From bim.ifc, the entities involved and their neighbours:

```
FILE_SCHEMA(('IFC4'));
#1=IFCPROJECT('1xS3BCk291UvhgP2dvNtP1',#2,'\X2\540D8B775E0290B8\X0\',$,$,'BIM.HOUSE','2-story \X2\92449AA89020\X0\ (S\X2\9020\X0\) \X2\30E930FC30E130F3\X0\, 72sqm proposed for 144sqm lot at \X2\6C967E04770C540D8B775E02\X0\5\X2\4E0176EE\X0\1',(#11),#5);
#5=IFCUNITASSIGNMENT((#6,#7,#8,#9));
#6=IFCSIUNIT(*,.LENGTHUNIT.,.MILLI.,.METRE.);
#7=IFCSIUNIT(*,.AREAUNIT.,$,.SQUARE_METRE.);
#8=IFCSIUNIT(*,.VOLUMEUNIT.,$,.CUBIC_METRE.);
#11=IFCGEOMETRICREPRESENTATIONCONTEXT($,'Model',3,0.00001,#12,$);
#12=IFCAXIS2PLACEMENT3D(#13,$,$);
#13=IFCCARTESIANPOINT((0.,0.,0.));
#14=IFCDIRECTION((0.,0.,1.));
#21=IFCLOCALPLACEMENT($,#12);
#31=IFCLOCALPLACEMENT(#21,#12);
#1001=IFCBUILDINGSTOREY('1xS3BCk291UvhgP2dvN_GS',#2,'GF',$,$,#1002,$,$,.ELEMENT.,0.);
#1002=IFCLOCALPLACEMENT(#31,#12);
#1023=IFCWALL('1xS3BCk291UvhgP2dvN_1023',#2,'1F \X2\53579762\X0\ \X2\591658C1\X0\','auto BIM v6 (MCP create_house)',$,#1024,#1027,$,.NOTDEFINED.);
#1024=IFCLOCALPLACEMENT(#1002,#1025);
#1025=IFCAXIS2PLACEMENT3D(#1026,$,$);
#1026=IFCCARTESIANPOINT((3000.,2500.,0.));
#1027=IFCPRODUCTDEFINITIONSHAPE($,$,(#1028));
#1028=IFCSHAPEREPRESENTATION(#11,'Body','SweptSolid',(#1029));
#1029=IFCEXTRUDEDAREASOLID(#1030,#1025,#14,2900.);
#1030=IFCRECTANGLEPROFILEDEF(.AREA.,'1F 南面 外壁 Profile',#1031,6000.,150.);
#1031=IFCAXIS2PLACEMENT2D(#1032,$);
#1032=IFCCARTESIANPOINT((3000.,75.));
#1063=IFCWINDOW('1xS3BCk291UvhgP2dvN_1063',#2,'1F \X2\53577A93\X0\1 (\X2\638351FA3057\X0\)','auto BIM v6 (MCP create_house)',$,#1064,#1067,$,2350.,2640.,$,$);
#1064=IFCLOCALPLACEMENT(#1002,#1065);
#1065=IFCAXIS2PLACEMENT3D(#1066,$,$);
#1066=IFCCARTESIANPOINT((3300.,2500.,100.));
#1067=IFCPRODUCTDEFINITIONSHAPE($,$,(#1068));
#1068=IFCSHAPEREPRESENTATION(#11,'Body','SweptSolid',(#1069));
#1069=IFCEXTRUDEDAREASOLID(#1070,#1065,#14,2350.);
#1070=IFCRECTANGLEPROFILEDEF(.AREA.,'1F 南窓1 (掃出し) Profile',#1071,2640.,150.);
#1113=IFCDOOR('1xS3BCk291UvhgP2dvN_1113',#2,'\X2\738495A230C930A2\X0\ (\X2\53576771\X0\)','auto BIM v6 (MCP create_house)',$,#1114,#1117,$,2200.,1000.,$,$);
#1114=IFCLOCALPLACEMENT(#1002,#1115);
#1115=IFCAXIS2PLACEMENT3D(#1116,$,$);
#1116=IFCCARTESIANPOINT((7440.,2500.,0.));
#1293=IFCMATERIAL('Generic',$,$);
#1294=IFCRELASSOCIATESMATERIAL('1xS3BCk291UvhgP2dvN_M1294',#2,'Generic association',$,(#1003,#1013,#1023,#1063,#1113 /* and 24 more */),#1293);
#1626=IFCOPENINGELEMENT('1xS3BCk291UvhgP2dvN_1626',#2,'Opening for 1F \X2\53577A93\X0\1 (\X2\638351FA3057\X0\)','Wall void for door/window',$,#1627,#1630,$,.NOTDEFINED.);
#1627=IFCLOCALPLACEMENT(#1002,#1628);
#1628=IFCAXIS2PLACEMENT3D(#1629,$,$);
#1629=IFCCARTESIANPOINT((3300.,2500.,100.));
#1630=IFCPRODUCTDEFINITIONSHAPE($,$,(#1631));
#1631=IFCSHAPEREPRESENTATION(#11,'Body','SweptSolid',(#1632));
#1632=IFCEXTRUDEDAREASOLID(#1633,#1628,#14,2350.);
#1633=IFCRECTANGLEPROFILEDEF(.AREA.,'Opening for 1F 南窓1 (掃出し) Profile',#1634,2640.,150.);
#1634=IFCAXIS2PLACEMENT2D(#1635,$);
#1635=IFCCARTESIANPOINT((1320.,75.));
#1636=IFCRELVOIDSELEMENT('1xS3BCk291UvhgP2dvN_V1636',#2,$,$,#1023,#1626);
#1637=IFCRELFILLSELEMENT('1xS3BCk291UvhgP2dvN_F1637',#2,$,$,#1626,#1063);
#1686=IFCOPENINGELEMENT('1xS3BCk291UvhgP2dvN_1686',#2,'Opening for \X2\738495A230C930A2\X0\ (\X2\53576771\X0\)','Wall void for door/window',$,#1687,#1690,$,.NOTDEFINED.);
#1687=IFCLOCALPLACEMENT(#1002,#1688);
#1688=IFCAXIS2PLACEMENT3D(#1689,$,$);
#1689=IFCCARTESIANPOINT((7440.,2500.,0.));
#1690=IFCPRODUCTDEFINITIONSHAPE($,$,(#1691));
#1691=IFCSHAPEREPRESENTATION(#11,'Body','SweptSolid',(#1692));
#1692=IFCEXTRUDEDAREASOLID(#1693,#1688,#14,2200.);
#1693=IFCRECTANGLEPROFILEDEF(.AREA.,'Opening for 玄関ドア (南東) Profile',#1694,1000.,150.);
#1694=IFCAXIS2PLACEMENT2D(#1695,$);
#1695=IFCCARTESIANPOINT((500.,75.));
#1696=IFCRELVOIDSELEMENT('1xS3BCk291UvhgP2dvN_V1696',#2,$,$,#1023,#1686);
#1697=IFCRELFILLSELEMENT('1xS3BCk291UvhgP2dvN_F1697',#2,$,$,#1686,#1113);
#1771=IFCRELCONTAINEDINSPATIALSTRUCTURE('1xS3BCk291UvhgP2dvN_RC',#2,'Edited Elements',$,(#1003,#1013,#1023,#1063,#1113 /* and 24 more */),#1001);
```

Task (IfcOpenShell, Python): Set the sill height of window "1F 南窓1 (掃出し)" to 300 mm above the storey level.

```python
import numpy as np
import ifcopenshell
import ifcopenshell.api.geometry
import ifcopenshell.geom
import ifcopenshell.util.element
import ifcopenshell.util.placement
import ifcopenshell.util.shape
import ifcopenshell.util.unit

model = ifcopenshell.open("bim.ifc")
unit_scale = ifcopenshell.util.unit.calculate_unit_scale(model)

window = model.by_guid("1xS3BCk291UvhgP2dvN_1063")
opening = window.FillsVoids[0].RelatingOpeningElement
storey = ifcopenshell.util.element.get_container(window, ifc_class="IfcBuildingStorey")
level = ifcopenshell.util.placement.get_local_placement(storey.ObjectPlacement)[2, 3]

# The opening's origin need not be at the sill, so measure its lowest point.
shape = ifcopenshell.geom.create_shape(ifcopenshell.geom.settings(), opening)
bottom = ifcopenshell.util.shape.get_shape_bottom_elevation(shape, shape.geometry) / unit_scale
dz = level + 300.0 - bottom

shift = np.array([0.0, 0.0, dz])
# The window is not placed relative to its opening, so move both.
for product in (opening, window):
    matrix = ifcopenshell.util.placement.get_local_placement(product.ObjectPlacement)
    matrix[:3, 3] += shift
    ifcopenshell.api.geometry.edit_object_placement(model, product=product, matrix=matrix, is_si=False)

print(f"moved by {dz * unit_scale:+.3f} m")

model.write("bim_v2.ifc")
```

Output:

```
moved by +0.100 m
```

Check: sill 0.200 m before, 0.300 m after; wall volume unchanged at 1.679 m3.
